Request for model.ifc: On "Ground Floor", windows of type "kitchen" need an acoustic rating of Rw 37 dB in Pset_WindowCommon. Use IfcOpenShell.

First a look at what the model holds.

```python
import ifcopenshell
import ifcopenshell.util.element

model = ifcopenshell.open("model.ifc")
print(model.schema)
storey = next(s for s in model.by_type("IfcBuildingStorey") if s.Name == "Ground Floor")
windows = [e for e in ifcopenshell.util.element.get_decomposition(storey) if e.is_a("IfcWindow")]
seen = {}
for e in windows:
    element_type = ifcopenshell.util.element.get_type(e)
    key = (element_type.Name if element_type != e and element_type else None, ifcopenshell.util.element.get_pset(e, "Pset_WindowCommon", "AcousticRating"))
    seen[key] = seen.get(key, 0) + 1
for (name, value), count in sorted(seen.items(), key=str):
    print(count, "x", name, "|", value)
```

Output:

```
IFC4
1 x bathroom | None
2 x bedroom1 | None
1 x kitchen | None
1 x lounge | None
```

```python
import ifcopenshell
import ifcopenshell.api.pset
import ifcopenshell.util.element

model = ifcopenshell.open("model.ifc")

storey = next(s for s in model.by_type("IfcBuildingStorey") if s.Name == "Ground Floor")
windows = [e for e in ifcopenshell.util.element.get_decomposition(storey) if e.is_a("IfcWindow")]

count = 0
for e in windows:
    element_type = ifcopenshell.util.element.get_type(e)
    if element_type in (None, e) or element_type.Name != "kitchen":
        continue
    # add_pset returns the element's existing set when there is one.
    pset = ifcopenshell.api.pset.add_pset(model, product=e, name="Pset_WindowCommon")
    ifcopenshell.api.pset.edit_pset(model, pset=pset, properties={"AcousticRating": "Rw 37 dB"})
    count += 1

print(count, "windows updated")

model.write("model_updated.ifc")
```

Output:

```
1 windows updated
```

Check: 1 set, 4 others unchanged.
